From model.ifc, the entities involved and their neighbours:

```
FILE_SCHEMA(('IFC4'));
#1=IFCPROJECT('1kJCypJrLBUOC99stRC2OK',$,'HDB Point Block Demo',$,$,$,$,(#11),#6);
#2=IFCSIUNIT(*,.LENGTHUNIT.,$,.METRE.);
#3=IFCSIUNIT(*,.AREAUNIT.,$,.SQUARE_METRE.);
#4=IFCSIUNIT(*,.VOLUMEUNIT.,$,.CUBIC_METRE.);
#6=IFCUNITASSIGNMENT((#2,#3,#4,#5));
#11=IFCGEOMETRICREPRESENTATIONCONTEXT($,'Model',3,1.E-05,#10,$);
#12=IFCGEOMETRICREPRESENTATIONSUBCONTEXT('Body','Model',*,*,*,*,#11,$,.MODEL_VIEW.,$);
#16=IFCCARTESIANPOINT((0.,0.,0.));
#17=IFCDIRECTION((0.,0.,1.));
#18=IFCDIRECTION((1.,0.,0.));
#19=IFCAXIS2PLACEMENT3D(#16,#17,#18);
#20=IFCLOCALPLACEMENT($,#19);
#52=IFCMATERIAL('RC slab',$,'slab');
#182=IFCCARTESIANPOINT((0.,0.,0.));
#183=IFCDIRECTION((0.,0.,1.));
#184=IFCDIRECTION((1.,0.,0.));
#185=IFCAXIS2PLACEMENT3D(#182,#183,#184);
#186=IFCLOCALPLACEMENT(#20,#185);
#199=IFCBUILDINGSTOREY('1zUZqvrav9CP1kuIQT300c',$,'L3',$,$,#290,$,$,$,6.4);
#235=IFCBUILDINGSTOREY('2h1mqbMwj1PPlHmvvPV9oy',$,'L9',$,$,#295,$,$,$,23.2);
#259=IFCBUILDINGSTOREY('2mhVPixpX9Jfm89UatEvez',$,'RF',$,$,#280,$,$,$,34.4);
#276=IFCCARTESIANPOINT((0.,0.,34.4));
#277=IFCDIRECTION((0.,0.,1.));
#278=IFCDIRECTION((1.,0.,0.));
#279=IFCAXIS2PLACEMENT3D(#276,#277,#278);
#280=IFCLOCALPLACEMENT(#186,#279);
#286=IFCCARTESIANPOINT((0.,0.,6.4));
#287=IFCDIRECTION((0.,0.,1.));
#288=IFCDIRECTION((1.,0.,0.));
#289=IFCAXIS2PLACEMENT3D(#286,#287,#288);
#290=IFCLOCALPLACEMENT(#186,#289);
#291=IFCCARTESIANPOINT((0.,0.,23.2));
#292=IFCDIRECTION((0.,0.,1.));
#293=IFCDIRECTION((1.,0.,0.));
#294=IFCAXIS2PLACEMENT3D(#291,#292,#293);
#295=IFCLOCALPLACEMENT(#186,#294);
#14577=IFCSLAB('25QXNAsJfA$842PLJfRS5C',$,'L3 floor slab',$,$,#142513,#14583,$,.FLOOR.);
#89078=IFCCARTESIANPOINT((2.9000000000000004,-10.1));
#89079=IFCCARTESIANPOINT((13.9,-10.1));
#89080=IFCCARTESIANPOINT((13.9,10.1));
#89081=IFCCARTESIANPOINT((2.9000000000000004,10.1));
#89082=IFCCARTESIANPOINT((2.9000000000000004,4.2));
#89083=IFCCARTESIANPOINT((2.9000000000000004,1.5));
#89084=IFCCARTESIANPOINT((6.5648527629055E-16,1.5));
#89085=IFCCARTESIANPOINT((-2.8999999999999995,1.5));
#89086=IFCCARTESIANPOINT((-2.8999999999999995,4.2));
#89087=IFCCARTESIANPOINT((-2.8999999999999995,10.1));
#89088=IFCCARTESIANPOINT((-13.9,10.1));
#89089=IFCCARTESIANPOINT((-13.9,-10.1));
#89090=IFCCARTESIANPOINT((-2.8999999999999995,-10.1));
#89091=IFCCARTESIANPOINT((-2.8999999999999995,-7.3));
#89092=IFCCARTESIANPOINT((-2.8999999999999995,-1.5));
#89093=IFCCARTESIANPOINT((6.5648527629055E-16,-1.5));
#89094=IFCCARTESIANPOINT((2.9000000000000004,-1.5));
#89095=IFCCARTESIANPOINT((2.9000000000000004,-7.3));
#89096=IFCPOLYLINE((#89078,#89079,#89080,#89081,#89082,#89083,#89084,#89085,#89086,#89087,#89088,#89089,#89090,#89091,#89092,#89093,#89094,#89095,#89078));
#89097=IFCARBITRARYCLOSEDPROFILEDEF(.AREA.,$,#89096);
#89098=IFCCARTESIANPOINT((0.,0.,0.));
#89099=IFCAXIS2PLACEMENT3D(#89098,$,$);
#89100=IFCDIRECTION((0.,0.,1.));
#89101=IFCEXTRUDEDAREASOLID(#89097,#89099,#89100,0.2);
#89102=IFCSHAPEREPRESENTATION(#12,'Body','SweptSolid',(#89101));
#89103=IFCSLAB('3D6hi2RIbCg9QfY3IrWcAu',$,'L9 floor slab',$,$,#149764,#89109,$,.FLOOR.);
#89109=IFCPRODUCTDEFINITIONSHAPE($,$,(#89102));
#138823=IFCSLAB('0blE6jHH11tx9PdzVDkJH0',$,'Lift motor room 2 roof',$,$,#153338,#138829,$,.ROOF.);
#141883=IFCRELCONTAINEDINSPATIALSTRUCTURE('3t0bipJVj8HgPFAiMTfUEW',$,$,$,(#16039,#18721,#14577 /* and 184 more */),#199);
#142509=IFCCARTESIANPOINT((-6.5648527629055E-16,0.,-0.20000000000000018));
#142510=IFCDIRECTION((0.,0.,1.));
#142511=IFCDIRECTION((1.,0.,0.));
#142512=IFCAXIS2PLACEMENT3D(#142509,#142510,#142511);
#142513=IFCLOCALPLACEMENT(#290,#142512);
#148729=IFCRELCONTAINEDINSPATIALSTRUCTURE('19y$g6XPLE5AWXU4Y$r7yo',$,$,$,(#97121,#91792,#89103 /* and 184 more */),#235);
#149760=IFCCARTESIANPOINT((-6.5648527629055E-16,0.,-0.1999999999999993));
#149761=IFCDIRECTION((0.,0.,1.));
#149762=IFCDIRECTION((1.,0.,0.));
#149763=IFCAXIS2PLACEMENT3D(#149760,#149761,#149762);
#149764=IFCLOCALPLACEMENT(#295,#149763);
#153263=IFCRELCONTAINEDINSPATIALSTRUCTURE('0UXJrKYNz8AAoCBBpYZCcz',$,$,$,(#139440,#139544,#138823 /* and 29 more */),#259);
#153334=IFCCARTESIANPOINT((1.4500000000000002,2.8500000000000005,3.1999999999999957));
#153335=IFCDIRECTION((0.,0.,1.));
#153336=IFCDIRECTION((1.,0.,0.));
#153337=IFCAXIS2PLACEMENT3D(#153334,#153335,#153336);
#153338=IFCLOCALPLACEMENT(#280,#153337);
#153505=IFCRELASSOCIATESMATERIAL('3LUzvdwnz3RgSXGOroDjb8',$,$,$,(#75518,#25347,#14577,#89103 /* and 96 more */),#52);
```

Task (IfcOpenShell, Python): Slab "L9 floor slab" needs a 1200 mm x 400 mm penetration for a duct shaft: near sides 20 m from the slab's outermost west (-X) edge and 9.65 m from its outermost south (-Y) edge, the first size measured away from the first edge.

```python
import numpy as np
import ifcopenshell
import ifcopenshell.api.feature
import ifcopenshell.api.geometry
import ifcopenshell.api.root
import ifcopenshell.geom
import ifcopenshell.util.placement
import ifcopenshell.util.representation
import ifcopenshell.util.shape
import ifcopenshell.util.unit

model = ifcopenshell.open("model.ifc")
unit_scale = ifcopenshell.util.unit.calculate_unit_scale(model)
settings = ifcopenshell.geom.settings()


def volume(element):
    """Net volume in cubic metres, openings subtracted."""
    shape = ifcopenshell.geom.create_shape(settings, element)
    return ifcopenshell.util.shape.get_volume(shape.geometry)


slab = model.by_guid("3D6hi2RIbCg9QfY3IrWcAu")
before = volume(slab)

# Extent in the slab's own axes, in metres. The edges named are its -X and -Y sides.
slab_shape = ifcopenshell.geom.create_shape(settings, slab)
vertices = ifcopenshell.util.shape.get_vertices(slab_shape.geometry)
x_min, y_min, bottom = vertices.min(axis=0)
top = vertices[:, 2].max()

opening = ifcopenshell.api.root.create_entity(model, ifc_class="IfcOpeningElement", name="Duct shaft opening", predefined_type="OPENING")
context = ifcopenshell.util.representation.get_context(model, "Model", "Body", "MODEL_VIEW")
width, depth = 1.2, 0.4
outline = [(0.0, 0.0), (width, 0.0), (width, depth), (0.0, depth), (0.0, 0.0)]
# Overshoot both faces by 50 mm so the cut is clean.
shape = ifcopenshell.api.geometry.add_slab_representation(
    model, context=context, depth=top - bottom + 0.1, polyline=outline
)
ifcopenshell.api.geometry.assign_representation(model, product=opening, representation=shape)

matrix = ifcopenshell.util.placement.get_local_placement(slab.ObjectPlacement)
matrix[:, 3] = matrix @ np.append(np.array([x_min + 20, y_min + 9.65, bottom - 0.05]) / unit_scale, 1.0)
ifcopenshell.api.geometry.edit_object_placement(model, product=opening, matrix=matrix, is_si=False)
ifcopenshell.api.feature.add_feature(model, feature=opening, element=slab)

after = volume(slab)

print(f"slab volume {before:.3f} -> {after:.3f} m3")

model.write("model_updated.ifc")
```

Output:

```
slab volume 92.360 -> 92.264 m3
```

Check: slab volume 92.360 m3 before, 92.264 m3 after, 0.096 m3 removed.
